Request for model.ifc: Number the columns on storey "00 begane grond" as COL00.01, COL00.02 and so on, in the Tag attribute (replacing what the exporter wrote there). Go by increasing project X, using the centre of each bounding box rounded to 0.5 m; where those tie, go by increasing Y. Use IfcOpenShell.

First a look at what the model holds.

```python
import ifcopenshell
import ifcopenshell.util.element
import ifcopenshell.util.placement

model = ifcopenshell.open("model.ifc")
print(model.schema)
storey = next(s for s in model.by_type("IfcBuildingStorey") if s.Name == "00 begane grond")
columns = [e for e in ifcopenshell.util.element.get_decomposition(storey) if e.is_a("IfcColumn")]
for e in sorted(columns, key=lambda e: e.id()):
    origin = ifcopenshell.util.placement.get_local_placement(e.ObjectPlacement)[:3, 3]
    print(e.id(), e.Tag, e.Name, origin.round(2) + 0.0, sep=" | ")
```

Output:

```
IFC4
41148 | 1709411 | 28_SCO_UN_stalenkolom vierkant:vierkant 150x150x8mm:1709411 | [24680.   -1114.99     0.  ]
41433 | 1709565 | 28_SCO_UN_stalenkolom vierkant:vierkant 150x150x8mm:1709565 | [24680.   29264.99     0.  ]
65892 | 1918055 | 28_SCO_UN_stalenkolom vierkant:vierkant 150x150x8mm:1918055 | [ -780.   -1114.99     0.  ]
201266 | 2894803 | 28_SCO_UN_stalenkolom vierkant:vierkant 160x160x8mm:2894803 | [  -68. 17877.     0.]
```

```python
import ifcopenshell
import ifcopenshell.geom
import ifcopenshell.util.element
import ifcopenshell.util.shape

model = ifcopenshell.open("model.ifc")
settings = ifcopenshell.geom.settings()
settings.set("use-world-coords", True)


def centre(element):
    shape = ifcopenshell.geom.create_shape(settings, element)
    return ifcopenshell.util.shape.get_bbox_centroid(shape.geometry)


storey = next(s for s in model.by_type("IfcBuildingStorey") if s.Name == "00 begane grond")
columns = [e for e in ifcopenshell.util.element.get_decomposition(storey) if e.is_a("IfcColumn")]

# Insertion points can sit at a corner or the storey origin, so sort by the geometry (in metres).
centres = {e: centre(e) for e in columns}
columns.sort(key=lambda e: (round(centres[e][0] / 0.5), centres[e][1]))

for i, e in enumerate(columns, start=1):
    number = f"COL00.{i:02d}"
    e.Tag = number
    print(e.id(), number)

model.write("model_rev.ifc")
```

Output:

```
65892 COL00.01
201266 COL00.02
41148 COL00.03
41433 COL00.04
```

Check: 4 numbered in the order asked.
